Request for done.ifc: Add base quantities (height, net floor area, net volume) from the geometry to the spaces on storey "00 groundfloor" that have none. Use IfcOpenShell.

First a look at what the model holds.

```python
import ifcopenshell
import ifcopenshell.util.element
import ifcopenshell.util.unit

model = ifcopenshell.open("done.ifc")
print(model.schema)
for unit_type in ("LENGTHUNIT", "AREAUNIT", "VOLUMEUNIT"):
    print(unit_type, ifcopenshell.util.unit.calculate_unit_scale(model, unit_type))
storey = next(s for s in model.by_type("IfcBuildingStorey") if s.Name == "00 groundfloor")
spaces = [e for e in ifcopenshell.util.element.get_decomposition(storey) if e.is_a("IfcSpace")]
for e in sorted(spaces, key=lambda e: e.id()):
    print(e.id(), e.is_a(), e.Name, list(ifcopenshell.util.element.get_psets(e, qtos_only=True)), sep=" | ")
```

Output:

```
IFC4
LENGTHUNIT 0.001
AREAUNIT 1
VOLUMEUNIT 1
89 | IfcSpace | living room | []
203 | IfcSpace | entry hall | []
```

```python
import ifcopenshell
import ifcopenshell.api.pset
import ifcopenshell.geom
import ifcopenshell.util.element
import ifcopenshell.util.shape
import ifcopenshell.util.unit

model = ifcopenshell.open("done.ifc")
unit_scale = ifcopenshell.util.unit.calculate_unit_scale(model)
area_scale = ifcopenshell.util.unit.calculate_unit_scale(model, "AREAUNIT")
volume_scale = ifcopenshell.util.unit.calculate_unit_scale(model, "VOLUMEUNIT")
settings = ifcopenshell.geom.settings()

storey = next(s for s in model.by_type("IfcBuildingStorey") if s.Name == "00 groundfloor")
spaces = [e for e in ifcopenshell.util.element.get_decomposition(storey) if e.is_a("IfcSpace")]

for e in sorted(spaces, key=lambda e: e.id()):
    if ifcopenshell.util.element.get_psets(e, qtos_only=True, should_inherit=False):
        continue
    # Geometry comes back in metres, in the element's own axes.
    shape = ifcopenshell.geom.create_shape(settings, e)
    values = {
        "Height": ifcopenshell.util.shape.get_z(shape.geometry) / unit_scale,
        "NetFloorArea": ifcopenshell.util.shape.get_footprint_area(shape.geometry) / area_scale,
        "NetVolume": ifcopenshell.util.shape.get_volume(shape.geometry) / volume_scale,
    }
    qto = ifcopenshell.api.pset.add_qto(model, product=e, name="Qto_SpaceBaseQuantities")
    ifcopenshell.api.pset.edit_qto(model, qto=qto, properties=values)
    print(e.id(), {k: round(v, 3) for k, v in values.items()})

model.write("done_updated.ifc")
```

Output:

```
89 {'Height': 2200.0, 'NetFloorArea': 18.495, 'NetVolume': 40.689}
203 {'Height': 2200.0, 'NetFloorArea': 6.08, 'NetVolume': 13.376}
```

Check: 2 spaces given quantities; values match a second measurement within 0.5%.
